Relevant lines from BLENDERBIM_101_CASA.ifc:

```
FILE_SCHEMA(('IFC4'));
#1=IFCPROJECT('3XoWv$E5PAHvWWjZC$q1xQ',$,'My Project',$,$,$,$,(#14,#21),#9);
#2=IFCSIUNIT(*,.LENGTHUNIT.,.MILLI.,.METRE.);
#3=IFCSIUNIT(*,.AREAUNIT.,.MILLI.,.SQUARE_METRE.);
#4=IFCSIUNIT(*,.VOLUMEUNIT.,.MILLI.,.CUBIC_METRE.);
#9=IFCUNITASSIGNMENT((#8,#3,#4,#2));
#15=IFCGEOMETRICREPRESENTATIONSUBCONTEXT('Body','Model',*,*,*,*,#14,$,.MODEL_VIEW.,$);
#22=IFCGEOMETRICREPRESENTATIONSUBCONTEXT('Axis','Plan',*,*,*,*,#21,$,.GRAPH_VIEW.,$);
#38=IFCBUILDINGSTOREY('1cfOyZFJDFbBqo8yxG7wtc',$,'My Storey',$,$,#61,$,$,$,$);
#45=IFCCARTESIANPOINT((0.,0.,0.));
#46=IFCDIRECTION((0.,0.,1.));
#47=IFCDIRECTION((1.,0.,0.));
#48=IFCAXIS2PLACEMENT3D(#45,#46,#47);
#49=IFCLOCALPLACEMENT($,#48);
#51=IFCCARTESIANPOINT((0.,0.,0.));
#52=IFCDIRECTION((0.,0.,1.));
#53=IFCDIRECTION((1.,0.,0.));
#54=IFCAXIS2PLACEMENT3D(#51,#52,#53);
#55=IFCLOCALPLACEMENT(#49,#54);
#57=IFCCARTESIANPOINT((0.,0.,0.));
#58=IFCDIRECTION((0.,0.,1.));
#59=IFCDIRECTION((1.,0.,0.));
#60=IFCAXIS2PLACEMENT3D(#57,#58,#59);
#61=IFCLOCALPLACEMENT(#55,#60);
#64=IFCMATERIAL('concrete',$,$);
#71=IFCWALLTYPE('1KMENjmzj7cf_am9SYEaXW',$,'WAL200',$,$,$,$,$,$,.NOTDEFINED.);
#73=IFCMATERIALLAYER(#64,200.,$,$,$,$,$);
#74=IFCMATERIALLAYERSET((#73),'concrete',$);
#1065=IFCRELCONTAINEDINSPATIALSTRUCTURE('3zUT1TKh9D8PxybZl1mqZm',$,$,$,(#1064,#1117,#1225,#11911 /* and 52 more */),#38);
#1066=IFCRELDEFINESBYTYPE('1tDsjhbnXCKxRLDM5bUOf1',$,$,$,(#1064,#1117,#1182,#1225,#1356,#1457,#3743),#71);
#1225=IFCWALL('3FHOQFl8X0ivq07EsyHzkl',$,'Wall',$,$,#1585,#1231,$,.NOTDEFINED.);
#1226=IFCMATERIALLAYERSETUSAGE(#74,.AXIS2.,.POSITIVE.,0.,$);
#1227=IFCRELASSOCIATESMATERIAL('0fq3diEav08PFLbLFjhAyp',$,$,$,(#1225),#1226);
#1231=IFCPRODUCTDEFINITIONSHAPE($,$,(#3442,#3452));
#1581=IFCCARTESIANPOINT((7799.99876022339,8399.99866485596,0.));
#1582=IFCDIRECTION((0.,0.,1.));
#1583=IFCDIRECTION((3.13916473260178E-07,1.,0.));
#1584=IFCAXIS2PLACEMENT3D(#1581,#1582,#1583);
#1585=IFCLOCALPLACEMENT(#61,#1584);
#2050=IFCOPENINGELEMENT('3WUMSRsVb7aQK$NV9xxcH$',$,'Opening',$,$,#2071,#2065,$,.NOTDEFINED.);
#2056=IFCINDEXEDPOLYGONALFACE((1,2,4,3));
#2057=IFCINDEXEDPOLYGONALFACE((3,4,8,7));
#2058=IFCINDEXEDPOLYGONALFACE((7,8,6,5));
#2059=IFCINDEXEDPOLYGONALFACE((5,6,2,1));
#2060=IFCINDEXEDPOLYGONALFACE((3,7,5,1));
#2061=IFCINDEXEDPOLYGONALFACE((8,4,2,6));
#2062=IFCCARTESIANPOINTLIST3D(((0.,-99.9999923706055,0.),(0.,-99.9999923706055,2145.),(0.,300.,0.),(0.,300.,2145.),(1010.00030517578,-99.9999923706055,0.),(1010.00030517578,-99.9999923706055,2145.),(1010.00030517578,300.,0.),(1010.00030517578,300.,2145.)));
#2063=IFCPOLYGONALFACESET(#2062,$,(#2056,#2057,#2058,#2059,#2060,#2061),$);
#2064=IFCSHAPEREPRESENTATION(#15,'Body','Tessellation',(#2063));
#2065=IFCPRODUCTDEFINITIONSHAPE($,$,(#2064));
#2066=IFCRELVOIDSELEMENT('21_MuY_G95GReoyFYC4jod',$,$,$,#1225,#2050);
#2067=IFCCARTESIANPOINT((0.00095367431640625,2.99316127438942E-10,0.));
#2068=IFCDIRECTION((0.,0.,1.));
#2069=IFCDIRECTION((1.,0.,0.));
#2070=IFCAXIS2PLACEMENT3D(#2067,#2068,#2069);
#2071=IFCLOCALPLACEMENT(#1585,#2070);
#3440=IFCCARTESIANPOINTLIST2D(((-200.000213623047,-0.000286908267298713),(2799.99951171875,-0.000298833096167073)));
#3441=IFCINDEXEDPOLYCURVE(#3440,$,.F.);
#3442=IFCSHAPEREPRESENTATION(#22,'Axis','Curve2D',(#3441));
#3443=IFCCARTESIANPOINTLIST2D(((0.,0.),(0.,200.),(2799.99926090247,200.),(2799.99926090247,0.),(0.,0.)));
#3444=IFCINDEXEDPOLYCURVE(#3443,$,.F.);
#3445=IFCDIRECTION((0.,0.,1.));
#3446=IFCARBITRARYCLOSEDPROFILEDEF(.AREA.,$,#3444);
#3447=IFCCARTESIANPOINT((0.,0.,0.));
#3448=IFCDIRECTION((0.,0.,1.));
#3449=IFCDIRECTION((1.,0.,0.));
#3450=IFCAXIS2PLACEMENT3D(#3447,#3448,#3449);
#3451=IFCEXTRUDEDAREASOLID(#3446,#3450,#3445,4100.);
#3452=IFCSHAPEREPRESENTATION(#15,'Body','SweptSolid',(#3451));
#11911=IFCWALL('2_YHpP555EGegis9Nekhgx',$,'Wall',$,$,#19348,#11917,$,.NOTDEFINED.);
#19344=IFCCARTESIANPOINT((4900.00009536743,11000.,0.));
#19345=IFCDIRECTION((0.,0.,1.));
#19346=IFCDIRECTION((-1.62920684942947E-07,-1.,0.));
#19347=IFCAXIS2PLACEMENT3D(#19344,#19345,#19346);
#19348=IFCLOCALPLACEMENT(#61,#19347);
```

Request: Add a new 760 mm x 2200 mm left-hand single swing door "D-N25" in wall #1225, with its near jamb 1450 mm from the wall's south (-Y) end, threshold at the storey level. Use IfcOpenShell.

```python
import numpy as np
import ifcopenshell
import ifcopenshell.api.feature
import ifcopenshell.api.geometry
import ifcopenshell.api.root
import ifcopenshell.api.spatial
import ifcopenshell.geom
import ifcopenshell.util.element
import ifcopenshell.util.placement
import ifcopenshell.util.representation
import ifcopenshell.util.shape
import ifcopenshell.util.unit

model = ifcopenshell.open("BLENDERBIM_101_CASA.ifc")
unit_scale = ifcopenshell.util.unit.calculate_unit_scale(model)
settings = ifcopenshell.geom.settings()


def volume(element):
    """Net volume in cubic metres, openings subtracted."""
    shape = ifcopenshell.geom.create_shape(settings, element)
    return ifcopenshell.util.shape.get_volume(shape.geometry)


wall = model.by_guid("3FHOQFl8X0ivq07EsyHzkl")
storey = ifcopenshell.util.element.get_container(wall, ifc_class="IfcBuildingStorey")
context = ifcopenshell.util.representation.get_context(model, "Model", "Body", "MODEL_VIEW")
before = volume(wall)

width, height, from_end, sill = 0.76, 2.2, 1.45, 0.0  # metres

# The wall runs along its own X axis, and the end named is its -X end.
wall_shape = ifcopenshell.geom.create_shape(settings, wall)
x, y, z = ifcopenshell.util.shape.get_vertices(wall_shape.geometry).T
start = x.min() + from_end
face, thickness = float(y.min()), float(y.max() - y.min())
wall_matrix = ifcopenshell.util.placement.get_local_placement(wall.ObjectPlacement)
level = ifcopenshell.util.placement.get_local_placement(storey.ObjectPlacement)[2, 3]


def in_wall(x, y):
    """Placement at x, y metres in the wall's axes, at sill height."""
    matrix = wall_matrix.copy()
    matrix[:, 3] = wall_matrix @ np.array([x / unit_scale, y / unit_scale, 0.0, 1.0])
    matrix[2, 3] = level + sill / unit_scale
    return matrix


# Opening: a box that overshoots both wall faces by 50 mm.
opening = ifcopenshell.api.root.create_entity(model, ifc_class="IfcOpeningElement", predefined_type="OPENING")
box = ifcopenshell.api.geometry.add_wall_representation(
    model, context=context, length=width, height=height, thickness=thickness + 0.1
)
ifcopenshell.api.geometry.assign_representation(model, product=opening, representation=box)
ifcopenshell.api.geometry.edit_object_placement(model, product=opening, matrix=in_wall(start, face - 0.05), is_si=False)
ifcopenshell.api.feature.add_feature(model, feature=opening, element=wall)

door = ifcopenshell.api.root.create_entity(model, ifc_class="IfcDoor", name="D-N25", predefined_type="DOOR")
door.OverallWidth, door.OverallHeight = width / unit_scale, height / unit_scale
door.OperationType = "SINGLE_SWING_LEFT"
body = ifcopenshell.api.geometry.add_door_representation(
    model,
    context=context,
    overall_width=door.OverallWidth,
    overall_height=door.OverallHeight,
    operation_type="SINGLE_SWING_LEFT",
    lining_properties={"LiningDepth": thickness / unit_scale, "ThresholdDepth": thickness / unit_scale},
)
ifcopenshell.api.geometry.assign_representation(model, product=door, representation=body)
ifcopenshell.api.spatial.assign_container(model, products=[door], relating_structure=storey)
ifcopenshell.api.feature.add_filling(model, opening=opening, element=door)

# The lining spans the wall, so the door starts at the wall face.
ifcopenshell.api.geometry.edit_object_placement(model, product=door, matrix=in_wall(start, face), is_si=False)

after = volume(wall)

print(f"wall volume {before:.3f} -> {after:.3f} m3")

model.write("BLENDERBIM_101_CASA_v2.ifc")
```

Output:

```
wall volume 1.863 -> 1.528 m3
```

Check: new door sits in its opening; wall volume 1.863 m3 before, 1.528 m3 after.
